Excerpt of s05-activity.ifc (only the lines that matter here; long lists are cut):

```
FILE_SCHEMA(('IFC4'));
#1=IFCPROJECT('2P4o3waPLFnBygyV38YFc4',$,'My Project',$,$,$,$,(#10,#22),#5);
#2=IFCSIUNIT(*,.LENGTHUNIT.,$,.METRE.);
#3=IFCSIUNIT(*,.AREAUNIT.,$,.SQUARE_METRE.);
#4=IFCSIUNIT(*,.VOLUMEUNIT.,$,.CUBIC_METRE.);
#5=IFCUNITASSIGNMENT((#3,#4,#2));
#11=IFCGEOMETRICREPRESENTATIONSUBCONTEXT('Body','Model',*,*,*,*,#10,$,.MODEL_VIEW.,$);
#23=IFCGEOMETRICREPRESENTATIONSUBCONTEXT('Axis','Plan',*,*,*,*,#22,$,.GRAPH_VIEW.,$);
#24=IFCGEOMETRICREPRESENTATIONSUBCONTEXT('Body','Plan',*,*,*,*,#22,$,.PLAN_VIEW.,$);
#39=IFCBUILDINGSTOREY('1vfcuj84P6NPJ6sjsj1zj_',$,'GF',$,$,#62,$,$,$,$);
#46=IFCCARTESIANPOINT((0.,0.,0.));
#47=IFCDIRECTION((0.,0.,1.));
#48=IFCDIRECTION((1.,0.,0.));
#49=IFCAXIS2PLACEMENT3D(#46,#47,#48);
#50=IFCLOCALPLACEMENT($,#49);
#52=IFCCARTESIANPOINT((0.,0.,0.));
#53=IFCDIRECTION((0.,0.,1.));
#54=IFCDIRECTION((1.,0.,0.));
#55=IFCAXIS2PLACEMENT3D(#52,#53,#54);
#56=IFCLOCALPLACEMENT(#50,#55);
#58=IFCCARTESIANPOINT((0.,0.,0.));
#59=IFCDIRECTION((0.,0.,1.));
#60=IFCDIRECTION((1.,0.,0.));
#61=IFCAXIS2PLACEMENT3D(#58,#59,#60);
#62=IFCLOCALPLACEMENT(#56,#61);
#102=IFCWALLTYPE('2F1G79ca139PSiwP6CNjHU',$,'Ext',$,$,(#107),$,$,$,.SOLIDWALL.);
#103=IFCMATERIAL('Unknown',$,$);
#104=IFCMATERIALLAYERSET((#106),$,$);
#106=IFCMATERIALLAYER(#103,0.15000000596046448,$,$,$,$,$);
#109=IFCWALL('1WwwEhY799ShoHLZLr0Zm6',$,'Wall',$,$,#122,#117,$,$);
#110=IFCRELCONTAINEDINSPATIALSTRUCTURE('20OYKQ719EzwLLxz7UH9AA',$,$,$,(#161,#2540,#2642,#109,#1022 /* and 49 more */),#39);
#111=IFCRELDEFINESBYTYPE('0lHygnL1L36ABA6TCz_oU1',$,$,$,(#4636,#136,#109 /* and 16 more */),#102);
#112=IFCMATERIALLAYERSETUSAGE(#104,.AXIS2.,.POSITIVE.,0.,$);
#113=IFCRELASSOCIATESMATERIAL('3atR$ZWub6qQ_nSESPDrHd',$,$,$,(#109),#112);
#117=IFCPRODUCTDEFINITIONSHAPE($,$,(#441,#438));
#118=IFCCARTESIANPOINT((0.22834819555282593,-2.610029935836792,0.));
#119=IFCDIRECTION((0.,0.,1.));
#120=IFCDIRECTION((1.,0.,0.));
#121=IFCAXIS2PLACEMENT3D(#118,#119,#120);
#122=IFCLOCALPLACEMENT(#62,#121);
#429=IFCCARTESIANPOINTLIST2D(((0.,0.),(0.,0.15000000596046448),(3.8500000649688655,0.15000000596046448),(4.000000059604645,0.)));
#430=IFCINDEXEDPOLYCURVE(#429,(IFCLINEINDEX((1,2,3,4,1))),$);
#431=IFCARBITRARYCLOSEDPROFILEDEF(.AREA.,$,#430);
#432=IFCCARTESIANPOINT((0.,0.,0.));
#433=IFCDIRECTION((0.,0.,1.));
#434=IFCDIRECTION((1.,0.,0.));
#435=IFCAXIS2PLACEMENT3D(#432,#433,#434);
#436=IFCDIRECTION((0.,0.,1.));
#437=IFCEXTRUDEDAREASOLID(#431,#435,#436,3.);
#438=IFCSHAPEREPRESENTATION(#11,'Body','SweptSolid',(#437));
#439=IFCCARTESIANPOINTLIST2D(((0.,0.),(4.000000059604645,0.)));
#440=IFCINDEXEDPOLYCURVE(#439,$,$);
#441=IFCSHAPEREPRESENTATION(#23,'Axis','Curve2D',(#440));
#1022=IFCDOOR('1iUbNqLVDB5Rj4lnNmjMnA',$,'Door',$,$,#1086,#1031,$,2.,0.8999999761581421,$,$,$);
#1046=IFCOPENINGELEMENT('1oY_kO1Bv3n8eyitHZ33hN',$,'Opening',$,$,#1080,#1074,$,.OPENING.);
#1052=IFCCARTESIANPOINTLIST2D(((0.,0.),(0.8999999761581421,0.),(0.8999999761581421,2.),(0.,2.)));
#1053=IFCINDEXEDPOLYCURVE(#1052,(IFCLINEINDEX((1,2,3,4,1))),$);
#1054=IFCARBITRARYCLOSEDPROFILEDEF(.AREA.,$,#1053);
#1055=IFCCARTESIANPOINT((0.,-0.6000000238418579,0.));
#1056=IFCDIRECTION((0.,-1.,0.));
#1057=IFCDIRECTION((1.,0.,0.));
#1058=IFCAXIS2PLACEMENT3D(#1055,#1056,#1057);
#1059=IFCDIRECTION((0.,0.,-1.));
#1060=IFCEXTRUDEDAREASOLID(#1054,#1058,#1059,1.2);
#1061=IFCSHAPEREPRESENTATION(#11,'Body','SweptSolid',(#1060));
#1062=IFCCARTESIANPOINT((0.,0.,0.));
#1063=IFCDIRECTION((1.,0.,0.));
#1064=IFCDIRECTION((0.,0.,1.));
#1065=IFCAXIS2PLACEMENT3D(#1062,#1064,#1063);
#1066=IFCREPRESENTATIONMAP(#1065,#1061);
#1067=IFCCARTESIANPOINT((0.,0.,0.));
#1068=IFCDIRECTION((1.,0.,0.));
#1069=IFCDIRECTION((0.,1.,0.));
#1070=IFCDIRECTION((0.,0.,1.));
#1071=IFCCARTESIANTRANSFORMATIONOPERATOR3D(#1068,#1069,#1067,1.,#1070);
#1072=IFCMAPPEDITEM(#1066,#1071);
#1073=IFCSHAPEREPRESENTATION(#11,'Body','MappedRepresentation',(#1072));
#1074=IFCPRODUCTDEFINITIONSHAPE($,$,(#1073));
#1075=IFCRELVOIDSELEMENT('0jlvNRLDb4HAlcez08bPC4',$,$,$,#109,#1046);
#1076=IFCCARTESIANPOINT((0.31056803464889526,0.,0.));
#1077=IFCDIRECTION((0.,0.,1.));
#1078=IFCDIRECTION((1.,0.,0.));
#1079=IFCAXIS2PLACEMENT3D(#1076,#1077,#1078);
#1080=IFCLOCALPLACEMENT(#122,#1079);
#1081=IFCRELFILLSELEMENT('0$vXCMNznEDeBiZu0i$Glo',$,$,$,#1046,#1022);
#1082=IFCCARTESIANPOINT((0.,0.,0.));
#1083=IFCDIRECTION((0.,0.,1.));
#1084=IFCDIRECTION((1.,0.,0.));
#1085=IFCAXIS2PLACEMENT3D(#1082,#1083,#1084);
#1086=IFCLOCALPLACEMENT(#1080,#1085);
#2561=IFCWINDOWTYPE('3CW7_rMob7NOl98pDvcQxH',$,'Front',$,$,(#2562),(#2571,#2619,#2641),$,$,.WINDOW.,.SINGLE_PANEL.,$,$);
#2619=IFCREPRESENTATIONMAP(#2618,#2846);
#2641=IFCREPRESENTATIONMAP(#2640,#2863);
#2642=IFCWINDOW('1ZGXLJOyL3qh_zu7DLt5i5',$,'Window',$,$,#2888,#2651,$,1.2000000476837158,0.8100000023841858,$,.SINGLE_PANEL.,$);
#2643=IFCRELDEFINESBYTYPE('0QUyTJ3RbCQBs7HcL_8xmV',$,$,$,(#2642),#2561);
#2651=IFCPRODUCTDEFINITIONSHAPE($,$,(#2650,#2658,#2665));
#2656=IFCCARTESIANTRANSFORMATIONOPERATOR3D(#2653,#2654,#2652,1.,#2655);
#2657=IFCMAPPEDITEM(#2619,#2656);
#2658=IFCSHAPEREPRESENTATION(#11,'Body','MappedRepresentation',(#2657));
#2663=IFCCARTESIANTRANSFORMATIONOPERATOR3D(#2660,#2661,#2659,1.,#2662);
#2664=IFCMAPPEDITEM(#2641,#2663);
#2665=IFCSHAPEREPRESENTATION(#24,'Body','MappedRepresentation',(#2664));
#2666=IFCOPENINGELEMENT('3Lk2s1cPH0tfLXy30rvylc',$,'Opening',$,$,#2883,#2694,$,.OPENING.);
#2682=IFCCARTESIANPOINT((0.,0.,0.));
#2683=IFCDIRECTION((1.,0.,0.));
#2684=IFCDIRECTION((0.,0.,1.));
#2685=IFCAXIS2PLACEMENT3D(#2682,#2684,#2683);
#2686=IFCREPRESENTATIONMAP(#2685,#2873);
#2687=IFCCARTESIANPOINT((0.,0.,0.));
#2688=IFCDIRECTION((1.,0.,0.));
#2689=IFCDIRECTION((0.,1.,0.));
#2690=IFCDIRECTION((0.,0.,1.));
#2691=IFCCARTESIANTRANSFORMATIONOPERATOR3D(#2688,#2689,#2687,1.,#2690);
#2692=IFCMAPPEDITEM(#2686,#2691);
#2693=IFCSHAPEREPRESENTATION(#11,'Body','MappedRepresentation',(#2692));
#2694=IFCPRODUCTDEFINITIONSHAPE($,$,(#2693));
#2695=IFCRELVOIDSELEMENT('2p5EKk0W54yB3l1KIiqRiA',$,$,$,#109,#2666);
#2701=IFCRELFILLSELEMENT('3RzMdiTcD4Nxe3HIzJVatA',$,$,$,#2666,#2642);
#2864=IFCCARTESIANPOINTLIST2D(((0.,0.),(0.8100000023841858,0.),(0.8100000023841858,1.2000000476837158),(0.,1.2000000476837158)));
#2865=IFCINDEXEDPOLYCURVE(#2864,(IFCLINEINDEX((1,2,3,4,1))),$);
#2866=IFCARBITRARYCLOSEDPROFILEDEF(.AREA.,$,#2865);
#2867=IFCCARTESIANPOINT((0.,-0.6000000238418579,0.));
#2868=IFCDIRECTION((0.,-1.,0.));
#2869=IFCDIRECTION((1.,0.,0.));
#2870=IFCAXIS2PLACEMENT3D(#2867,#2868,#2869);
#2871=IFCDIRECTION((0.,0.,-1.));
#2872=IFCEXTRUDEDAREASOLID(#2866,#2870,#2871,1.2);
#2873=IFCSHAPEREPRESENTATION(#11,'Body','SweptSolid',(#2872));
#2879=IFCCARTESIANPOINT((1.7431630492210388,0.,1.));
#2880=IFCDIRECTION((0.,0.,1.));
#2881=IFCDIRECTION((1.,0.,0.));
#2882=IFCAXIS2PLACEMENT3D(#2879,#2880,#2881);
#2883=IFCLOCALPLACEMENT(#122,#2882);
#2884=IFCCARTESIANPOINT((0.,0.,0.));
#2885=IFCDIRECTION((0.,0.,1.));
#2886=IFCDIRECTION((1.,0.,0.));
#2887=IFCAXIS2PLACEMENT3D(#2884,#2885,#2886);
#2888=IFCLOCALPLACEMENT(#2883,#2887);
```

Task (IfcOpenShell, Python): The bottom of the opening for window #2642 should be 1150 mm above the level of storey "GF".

```python
import numpy as np
import ifcopenshell
import ifcopenshell.api.geometry
import ifcopenshell.geom
import ifcopenshell.util.element
import ifcopenshell.util.placement
import ifcopenshell.util.shape
import ifcopenshell.util.unit

model = ifcopenshell.open("s05-activity.ifc")
unit_scale = ifcopenshell.util.unit.calculate_unit_scale(model)

window = model.by_guid("1ZGXLJOyL3qh_zu7DLt5i5")
opening = window.FillsVoids[0].RelatingOpeningElement
storey = ifcopenshell.util.element.get_container(window, ifc_class="IfcBuildingStorey")
level = ifcopenshell.util.placement.get_local_placement(storey.ObjectPlacement)[2, 3]

# The opening's origin need not be at the sill, so measure its lowest point.
shape = ifcopenshell.geom.create_shape(ifcopenshell.geom.settings(), opening)
bottom = ifcopenshell.util.shape.get_shape_bottom_elevation(shape, shape.geometry) / unit_scale
dz = level + 1.15 - bottom

shift = np.array([0.0, 0.0, dz])
# The window is placed relative to its opening, so it follows when the opening moves.
matrix = ifcopenshell.util.placement.get_local_placement(opening.ObjectPlacement)
matrix[:3, 3] += shift
ifcopenshell.api.geometry.edit_object_placement(
    model, product=opening, matrix=matrix, is_si=False, should_transform_children=True
)

print(f"moved by {dz * unit_scale:+.3f} m")

model.write("s05-activity_v2.ifc")
```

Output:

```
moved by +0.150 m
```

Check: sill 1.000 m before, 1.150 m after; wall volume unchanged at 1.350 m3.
